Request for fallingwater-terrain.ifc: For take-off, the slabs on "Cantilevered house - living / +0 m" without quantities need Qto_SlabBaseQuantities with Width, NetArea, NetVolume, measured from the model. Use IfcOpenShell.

First a look at what the model holds.

```python
import ifcopenshell
import ifcopenshell.util.element
import ifcopenshell.util.unit

model = ifcopenshell.open("fallingwater-terrain.ifc")
print(model.schema)
for unit_type in ("LENGTHUNIT", "AREAUNIT", "VOLUMEUNIT"):
    print(unit_type, ifcopenshell.util.unit.calculate_unit_scale(model, unit_type))
storey = next(s for s in model.by_type("IfcBuildingStorey") if s.Name == "Cantilevered house - living / +0 m")
slabs = [e for e in ifcopenshell.util.element.get_decomposition(storey) if e.is_a("IfcSlab")]
for e in sorted(slabs, key=lambda e: e.id()):
    print(e.id(), e.is_a(), e.Name, list(ifcopenshell.util.element.get_psets(e, qtos_only=True)), sep=" | ")
```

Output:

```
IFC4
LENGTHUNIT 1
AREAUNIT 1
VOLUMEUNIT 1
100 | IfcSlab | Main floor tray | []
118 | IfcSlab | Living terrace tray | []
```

```python
import ifcopenshell
import ifcopenshell.api.pset
import ifcopenshell.geom
import ifcopenshell.util.element
import ifcopenshell.util.shape
import ifcopenshell.util.unit

model = ifcopenshell.open("fallingwater-terrain.ifc")
unit_scale = ifcopenshell.util.unit.calculate_unit_scale(model)
area_scale = ifcopenshell.util.unit.calculate_unit_scale(model, "AREAUNIT")
volume_scale = ifcopenshell.util.unit.calculate_unit_scale(model, "VOLUMEUNIT")
settings = ifcopenshell.geom.settings()

storey = next(s for s in model.by_type("IfcBuildingStorey") if s.Name == "Cantilevered house - living / +0 m")
slabs = [e for e in ifcopenshell.util.element.get_decomposition(storey) if e.is_a("IfcSlab")]

for e in sorted(slabs, key=lambda e: e.id()):
    if ifcopenshell.util.element.get_psets(e, qtos_only=True, should_inherit=False):
        continue
    # Geometry comes back in metres, in the element's own axes.
    shape = ifcopenshell.geom.create_shape(settings, e)
    values = {
        "Width": ifcopenshell.util.shape.get_z(shape.geometry) / unit_scale,
        "NetArea": ifcopenshell.util.shape.get_footprint_area(shape.geometry) / area_scale,
        "NetVolume": ifcopenshell.util.shape.get_volume(shape.geometry) / volume_scale,
    }
    qto = ifcopenshell.api.pset.add_qto(model, product=e, name="Qto_SlabBaseQuantities")
    ifcopenshell.api.pset.edit_qto(model, qto=qto, properties=values)
    print(e.id(), {k: round(v, 3) for k, v in values.items()})

model.write("fallingwater-terrain_v2.ifc")
```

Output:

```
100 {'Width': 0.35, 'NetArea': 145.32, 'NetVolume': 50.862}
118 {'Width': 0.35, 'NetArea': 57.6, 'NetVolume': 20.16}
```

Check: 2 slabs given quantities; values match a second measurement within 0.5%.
